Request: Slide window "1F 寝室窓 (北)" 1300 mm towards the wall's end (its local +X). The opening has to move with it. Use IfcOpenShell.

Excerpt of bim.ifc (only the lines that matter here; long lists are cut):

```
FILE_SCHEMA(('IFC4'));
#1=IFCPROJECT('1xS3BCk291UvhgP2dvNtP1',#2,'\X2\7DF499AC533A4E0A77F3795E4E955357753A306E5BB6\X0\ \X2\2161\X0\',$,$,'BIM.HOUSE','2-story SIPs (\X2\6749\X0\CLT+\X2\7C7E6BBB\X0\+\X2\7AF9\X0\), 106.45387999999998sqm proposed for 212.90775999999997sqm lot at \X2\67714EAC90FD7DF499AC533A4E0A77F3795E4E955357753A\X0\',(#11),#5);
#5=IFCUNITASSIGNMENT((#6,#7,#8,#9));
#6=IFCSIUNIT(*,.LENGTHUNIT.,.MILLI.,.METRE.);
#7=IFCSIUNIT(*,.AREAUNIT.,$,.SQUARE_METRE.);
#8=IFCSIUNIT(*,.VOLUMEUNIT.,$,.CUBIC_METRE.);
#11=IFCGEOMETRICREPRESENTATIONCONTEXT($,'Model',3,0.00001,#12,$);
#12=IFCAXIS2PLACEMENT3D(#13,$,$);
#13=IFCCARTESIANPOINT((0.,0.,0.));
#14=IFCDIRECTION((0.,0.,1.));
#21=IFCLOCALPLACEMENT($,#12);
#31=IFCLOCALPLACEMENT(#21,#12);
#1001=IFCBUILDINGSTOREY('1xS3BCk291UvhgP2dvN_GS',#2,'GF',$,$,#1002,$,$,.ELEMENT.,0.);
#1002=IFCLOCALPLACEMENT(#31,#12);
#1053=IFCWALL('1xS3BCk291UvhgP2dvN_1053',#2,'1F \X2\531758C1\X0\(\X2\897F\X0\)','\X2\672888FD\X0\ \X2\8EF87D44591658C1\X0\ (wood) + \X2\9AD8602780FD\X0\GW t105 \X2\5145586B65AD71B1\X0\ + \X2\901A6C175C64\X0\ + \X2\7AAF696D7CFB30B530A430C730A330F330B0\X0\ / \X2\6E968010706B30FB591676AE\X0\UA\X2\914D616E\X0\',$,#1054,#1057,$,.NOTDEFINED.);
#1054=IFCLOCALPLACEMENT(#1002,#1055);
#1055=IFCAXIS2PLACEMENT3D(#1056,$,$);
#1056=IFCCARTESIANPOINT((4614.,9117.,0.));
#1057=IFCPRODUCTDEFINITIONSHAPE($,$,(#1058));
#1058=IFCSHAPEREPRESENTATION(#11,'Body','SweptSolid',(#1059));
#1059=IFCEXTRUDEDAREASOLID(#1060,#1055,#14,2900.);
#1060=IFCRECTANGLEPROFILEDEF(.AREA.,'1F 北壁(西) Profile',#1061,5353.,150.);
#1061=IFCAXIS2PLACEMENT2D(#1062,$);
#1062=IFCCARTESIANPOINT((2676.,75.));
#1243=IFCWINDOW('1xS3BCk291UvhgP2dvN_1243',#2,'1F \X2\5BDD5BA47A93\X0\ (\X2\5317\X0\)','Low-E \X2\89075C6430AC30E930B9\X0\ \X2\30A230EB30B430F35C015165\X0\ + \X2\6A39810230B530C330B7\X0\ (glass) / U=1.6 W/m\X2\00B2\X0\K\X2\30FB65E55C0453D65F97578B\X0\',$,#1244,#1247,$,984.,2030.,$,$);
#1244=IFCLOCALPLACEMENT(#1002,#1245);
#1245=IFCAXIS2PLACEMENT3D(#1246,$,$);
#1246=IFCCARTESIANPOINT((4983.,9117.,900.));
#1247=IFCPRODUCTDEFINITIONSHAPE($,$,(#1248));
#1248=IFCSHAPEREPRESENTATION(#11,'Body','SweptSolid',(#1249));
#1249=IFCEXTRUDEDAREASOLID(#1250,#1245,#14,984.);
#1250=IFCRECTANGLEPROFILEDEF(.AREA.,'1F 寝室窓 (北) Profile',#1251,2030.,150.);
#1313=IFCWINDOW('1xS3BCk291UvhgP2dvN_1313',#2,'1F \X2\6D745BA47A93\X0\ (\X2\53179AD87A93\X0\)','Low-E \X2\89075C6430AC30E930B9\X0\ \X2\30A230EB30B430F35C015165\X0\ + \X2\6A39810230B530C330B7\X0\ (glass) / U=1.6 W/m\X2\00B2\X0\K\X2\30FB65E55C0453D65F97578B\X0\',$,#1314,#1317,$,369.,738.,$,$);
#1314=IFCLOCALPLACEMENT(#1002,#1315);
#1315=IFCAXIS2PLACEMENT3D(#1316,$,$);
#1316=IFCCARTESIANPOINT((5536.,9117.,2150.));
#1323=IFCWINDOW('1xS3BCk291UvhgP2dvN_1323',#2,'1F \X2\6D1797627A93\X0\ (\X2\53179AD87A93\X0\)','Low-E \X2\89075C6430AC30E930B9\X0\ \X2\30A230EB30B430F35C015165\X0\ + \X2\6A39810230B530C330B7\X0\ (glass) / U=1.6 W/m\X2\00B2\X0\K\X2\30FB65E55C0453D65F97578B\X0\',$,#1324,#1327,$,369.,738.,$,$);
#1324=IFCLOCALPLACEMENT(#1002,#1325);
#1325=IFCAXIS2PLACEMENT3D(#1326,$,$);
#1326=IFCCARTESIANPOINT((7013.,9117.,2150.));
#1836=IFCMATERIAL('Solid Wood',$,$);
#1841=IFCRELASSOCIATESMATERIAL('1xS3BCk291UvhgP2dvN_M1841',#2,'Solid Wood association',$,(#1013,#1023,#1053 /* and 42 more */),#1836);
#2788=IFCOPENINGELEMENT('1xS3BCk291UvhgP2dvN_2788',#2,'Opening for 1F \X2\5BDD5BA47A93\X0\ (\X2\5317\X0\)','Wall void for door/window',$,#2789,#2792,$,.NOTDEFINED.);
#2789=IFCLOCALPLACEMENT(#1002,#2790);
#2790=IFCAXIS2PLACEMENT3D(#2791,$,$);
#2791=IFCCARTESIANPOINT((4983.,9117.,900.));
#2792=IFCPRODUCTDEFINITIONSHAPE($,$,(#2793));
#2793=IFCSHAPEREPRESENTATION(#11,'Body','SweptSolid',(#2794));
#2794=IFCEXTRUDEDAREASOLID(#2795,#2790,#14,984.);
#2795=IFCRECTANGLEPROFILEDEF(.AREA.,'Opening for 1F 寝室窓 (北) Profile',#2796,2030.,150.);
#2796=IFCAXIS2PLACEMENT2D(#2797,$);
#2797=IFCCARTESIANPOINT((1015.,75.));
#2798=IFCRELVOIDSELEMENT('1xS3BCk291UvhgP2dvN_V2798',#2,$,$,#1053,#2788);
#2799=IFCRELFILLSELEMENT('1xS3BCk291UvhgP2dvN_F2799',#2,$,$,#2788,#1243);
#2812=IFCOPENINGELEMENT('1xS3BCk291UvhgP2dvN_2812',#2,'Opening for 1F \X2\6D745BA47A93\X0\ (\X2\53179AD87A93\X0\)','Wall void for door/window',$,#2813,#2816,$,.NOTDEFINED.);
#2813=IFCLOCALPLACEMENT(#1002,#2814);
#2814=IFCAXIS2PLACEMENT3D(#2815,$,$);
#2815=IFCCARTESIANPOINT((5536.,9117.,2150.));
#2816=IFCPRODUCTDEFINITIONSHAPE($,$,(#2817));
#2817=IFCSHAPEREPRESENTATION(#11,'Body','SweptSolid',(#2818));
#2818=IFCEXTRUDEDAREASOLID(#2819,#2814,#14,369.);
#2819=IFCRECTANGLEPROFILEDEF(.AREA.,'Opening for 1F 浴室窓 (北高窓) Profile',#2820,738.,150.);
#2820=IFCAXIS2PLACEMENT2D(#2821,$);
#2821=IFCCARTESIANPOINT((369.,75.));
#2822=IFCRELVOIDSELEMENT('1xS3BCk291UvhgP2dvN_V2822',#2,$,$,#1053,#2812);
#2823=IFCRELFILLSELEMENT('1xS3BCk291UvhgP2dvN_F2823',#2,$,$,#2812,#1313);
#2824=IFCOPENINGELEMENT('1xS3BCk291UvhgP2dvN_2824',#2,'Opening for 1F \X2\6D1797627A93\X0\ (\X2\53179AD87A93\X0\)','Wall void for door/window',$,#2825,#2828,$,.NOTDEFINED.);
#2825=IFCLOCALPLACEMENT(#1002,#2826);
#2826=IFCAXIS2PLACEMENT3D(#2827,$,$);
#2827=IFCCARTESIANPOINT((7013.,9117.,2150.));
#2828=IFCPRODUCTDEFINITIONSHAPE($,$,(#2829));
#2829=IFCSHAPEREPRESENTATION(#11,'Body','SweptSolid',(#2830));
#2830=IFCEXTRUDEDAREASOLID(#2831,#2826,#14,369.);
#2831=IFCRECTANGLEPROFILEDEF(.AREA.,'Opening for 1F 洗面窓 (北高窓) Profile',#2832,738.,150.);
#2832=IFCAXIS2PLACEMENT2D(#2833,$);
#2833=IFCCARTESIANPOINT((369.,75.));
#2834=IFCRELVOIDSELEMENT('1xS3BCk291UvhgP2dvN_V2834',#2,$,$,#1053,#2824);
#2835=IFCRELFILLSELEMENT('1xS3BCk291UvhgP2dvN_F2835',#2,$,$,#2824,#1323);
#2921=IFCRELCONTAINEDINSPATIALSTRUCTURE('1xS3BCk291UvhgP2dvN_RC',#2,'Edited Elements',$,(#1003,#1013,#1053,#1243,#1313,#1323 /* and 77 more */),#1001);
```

```python
import ifcopenshell
import ifcopenshell.api.geometry
import ifcopenshell.util.placement

model = ifcopenshell.open("bim.ifc")

window = model.by_id(1243)
opening = window.FillsVoids[0].RelatingOpeningElement
wall = opening.VoidsElements[0].RelatingBuildingElement

wall_matrix = ifcopenshell.util.placement.get_local_placement(wall.ObjectPlacement)
shift = wall_matrix[:3, 0] * 1300.0
before = ifcopenshell.util.placement.get_local_placement(window.ObjectPlacement)[:3, 3].copy()

# The window is not placed relative to its opening, so move both.
for product in (opening, window):
    matrix = ifcopenshell.util.placement.get_local_placement(product.ObjectPlacement)
    matrix[:3, 3] += shift
    ifcopenshell.api.geometry.edit_object_placement(model, product=product, matrix=matrix, is_si=False)

after = ifcopenshell.util.placement.get_local_placement(window.ObjectPlacement)[:3, 3]
print("window moved by", (after - before).round(3) + 0.0)

model.write("bim_updated.ifc")
```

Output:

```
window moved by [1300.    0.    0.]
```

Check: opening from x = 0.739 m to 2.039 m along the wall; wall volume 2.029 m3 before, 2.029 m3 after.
